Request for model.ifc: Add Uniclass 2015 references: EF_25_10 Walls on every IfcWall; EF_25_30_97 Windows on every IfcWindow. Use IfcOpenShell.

First a look at what the model holds.

```python
import ifcopenshell

model = ifcopenshell.open("model.ifc")
print(model.schema)
print("classifications:", [c.Name for c in model.by_type("IfcClassification")])
for ifc_class in ("IfcDoor", "IfcRoof", "IfcStair", "IfcWall", "IfcWindow"):
    print(ifc_class, len(model.by_type(ifc_class)))
```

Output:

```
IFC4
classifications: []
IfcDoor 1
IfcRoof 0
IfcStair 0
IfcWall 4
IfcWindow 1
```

```python
import ifcopenshell
import ifcopenshell.api.classification

model = ifcopenshell.open("model.ifc")

system = ifcopenshell.api.classification.add_classification(model, classification="Uniclass 2015")

codes = {
    "IfcWall": ("EF_25_10", "Walls"),
    "IfcWindow": ("EF_25_30_97", "Windows"),
}
for ifc_class, (code, name) in codes.items():
    products = model.by_type(ifc_class)
    ifcopenshell.api.classification.add_reference(
        model, products=products, classification=system, identification=code, name=name
    )
    print(code, len(products))

model.write("model_v2.ifc")
```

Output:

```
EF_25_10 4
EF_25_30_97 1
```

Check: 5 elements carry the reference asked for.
